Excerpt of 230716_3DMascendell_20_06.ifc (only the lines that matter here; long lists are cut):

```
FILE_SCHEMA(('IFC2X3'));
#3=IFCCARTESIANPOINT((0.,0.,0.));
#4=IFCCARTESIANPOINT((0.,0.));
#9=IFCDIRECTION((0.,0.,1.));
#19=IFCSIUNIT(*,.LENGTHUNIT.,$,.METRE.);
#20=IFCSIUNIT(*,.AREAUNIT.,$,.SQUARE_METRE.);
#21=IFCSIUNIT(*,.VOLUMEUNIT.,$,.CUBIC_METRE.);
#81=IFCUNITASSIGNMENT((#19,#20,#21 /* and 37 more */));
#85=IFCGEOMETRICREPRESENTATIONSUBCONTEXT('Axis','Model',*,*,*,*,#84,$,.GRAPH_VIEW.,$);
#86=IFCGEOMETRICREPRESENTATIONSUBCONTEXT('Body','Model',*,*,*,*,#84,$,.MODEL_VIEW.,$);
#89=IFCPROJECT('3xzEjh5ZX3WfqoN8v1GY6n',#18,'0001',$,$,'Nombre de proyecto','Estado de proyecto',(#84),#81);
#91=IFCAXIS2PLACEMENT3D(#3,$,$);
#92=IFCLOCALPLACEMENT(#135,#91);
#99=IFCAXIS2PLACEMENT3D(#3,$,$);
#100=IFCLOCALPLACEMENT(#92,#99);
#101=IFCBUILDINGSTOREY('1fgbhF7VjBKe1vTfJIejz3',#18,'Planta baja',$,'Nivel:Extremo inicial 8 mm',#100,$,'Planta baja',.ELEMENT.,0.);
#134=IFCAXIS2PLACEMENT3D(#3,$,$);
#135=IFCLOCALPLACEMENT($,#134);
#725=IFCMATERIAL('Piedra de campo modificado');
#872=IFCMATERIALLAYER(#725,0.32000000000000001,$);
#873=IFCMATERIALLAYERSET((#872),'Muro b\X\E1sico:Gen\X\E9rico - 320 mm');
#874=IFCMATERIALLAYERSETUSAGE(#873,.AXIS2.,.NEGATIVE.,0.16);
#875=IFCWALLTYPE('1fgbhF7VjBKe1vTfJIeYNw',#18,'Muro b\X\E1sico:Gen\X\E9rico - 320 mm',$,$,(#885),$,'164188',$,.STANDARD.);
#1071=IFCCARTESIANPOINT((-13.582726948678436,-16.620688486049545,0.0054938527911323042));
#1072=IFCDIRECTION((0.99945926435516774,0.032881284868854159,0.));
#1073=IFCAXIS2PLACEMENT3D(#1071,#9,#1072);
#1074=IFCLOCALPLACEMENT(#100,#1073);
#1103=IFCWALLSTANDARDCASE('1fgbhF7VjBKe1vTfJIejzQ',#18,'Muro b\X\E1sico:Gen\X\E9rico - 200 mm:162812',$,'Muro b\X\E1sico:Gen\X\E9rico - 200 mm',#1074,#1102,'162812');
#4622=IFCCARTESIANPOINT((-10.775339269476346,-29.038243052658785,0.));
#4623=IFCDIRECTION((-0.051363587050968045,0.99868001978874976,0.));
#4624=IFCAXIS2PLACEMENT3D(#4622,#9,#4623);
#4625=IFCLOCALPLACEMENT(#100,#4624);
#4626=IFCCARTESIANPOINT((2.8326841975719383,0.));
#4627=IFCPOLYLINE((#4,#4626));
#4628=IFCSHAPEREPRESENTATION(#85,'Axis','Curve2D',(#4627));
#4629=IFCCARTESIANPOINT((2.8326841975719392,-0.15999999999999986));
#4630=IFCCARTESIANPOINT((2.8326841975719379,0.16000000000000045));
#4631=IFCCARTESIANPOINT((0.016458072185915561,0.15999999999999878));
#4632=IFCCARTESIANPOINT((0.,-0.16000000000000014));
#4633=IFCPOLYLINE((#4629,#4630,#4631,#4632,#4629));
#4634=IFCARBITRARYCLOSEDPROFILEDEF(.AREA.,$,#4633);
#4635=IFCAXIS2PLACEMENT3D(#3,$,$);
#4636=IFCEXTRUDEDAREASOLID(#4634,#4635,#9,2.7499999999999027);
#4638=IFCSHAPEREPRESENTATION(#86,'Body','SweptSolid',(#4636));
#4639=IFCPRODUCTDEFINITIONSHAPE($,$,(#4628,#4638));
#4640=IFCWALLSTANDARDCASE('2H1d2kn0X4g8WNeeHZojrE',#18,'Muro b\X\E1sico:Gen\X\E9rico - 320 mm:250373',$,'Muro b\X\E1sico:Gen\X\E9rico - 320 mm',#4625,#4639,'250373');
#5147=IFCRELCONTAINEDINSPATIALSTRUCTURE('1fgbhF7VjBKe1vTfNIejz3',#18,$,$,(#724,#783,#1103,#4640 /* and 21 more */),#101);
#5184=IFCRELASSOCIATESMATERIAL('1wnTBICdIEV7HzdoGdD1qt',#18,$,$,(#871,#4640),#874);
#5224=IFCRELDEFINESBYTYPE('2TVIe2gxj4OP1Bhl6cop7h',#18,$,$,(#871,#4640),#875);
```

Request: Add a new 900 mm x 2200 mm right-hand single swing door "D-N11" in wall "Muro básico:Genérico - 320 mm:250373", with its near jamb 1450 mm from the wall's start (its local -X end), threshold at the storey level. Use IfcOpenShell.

```python
import numpy as np
import ifcopenshell
import ifcopenshell.api.feature
import ifcopenshell.api.geometry
import ifcopenshell.api.root
import ifcopenshell.api.spatial
import ifcopenshell.api.type
import ifcopenshell.geom
import ifcopenshell.util.element
import ifcopenshell.util.placement
import ifcopenshell.util.representation
import ifcopenshell.util.shape
import ifcopenshell.util.unit

model = ifcopenshell.open("230716_3DMascendell_20_06.ifc")
unit_scale = ifcopenshell.util.unit.calculate_unit_scale(model)
settings = ifcopenshell.geom.settings()


def volume(element):
    """Net volume in cubic metres, openings subtracted."""
    shape = ifcopenshell.geom.create_shape(settings, element)
    return ifcopenshell.util.shape.get_volume(shape.geometry)


wall = model.by_guid("2H1d2kn0X4g8WNeeHZojrE")
storey = ifcopenshell.util.element.get_container(wall, ifc_class="IfcBuildingStorey")
context = ifcopenshell.util.representation.get_context(model, "Model", "Body", "MODEL_VIEW")
before = volume(wall)

width, height, from_end, sill = 0.9, 2.2, 1.45, 0.0  # metres

# The wall runs along its own X axis, and the end named is its -X end.
wall_shape = ifcopenshell.geom.create_shape(settings, wall)
x, y, z = ifcopenshell.util.shape.get_vertices(wall_shape.geometry).T
start = x.min() + from_end
face, thickness = float(y.min()), float(y.max() - y.min())
wall_matrix = ifcopenshell.util.placement.get_local_placement(wall.ObjectPlacement)
level = ifcopenshell.util.placement.get_local_placement(storey.ObjectPlacement)[2, 3]


def in_wall(x, y):
    """Placement at x, y metres in the wall's axes, at sill height."""
    matrix = wall_matrix.copy()
    matrix[:, 3] = wall_matrix @ np.array([x / unit_scale, y / unit_scale, 0.0, 1.0])
    matrix[2, 3] = level + sill / unit_scale
    return matrix


# Opening: a box that overshoots both wall faces by 50 mm.
opening = ifcopenshell.api.root.create_entity(model, ifc_class="IfcOpeningElement")
box = ifcopenshell.api.geometry.add_wall_representation(
    model, context=context, length=width, height=height, thickness=thickness + 0.1
)
ifcopenshell.api.geometry.assign_representation(model, product=opening, representation=box)
ifcopenshell.api.geometry.edit_object_placement(model, product=opening, matrix=in_wall(start, face - 0.05), is_si=False)
ifcopenshell.api.feature.add_feature(model, feature=opening, element=wall)

door = ifcopenshell.api.root.create_entity(model, ifc_class="IfcDoor", name="D-N11")
door.OverallWidth, door.OverallHeight = width / unit_scale, height / unit_scale
body = ifcopenshell.api.geometry.add_door_representation(
    model,
    context=context,
    overall_width=door.OverallWidth,
    overall_height=door.OverallHeight,
    operation_type="SINGLE_SWING_RIGHT",
    lining_properties={"LiningDepth": thickness / unit_scale, "ThresholdDepth": thickness / unit_scale},
)
ifcopenshell.api.geometry.assign_representation(model, product=door, representation=body)
ifcopenshell.api.spatial.assign_container(model, products=[door], relating_structure=storey)
fills = ifcopenshell.api.feature.add_filling(model, opening=opening, element=door)
fills.OwnerHistory = door.OwnerHistory  # required in IFC2X3

# IFC2X3 keeps the operation on the door style.
style = ifcopenshell.api.root.create_entity(model, ifc_class="IfcDoorStyle", name="D-N11")
style.OperationType, style.ConstructionType = "SINGLE_SWING_RIGHT", "NOTDEFINED"
style.ParameterTakesPrecedence = style.Sizeable = False
ifcopenshell.api.type.assign_type(model, related_objects=[door], relating_type=style)

# The lining spans the wall, so the door starts at the wall face.
ifcopenshell.api.geometry.edit_object_placement(model, product=door, matrix=in_wall(start, face), is_si=False)

after = volume(wall)

print(f"wall volume {before:.3f} -> {after:.3f} m3")

model.write("230716_3DMascendell_20_06_updated.ifc")
```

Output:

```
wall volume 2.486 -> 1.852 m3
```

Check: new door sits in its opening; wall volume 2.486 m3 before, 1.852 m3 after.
